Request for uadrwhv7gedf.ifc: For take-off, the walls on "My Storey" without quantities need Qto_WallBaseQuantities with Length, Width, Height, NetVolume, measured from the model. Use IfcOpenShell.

First a look at what the model holds.

```python
import ifcopenshell
import ifcopenshell.util.element
import ifcopenshell.util.unit

model = ifcopenshell.open("uadrwhv7gedf.ifc")
print(model.schema)
for unit_type in ("LENGTHUNIT", "AREAUNIT", "VOLUMEUNIT"):
    print(unit_type, ifcopenshell.util.unit.calculate_unit_scale(model, unit_type))
storey = next(s for s in model.by_type("IfcBuildingStorey") if s.Name == "My Storey")
walls = [e for e in ifcopenshell.util.element.get_decomposition(storey) if e.is_a("IfcWall")]
for e in sorted(walls, key=lambda e: e.id()):
    print(e.id(), e.is_a(), e.Name, list(ifcopenshell.util.element.get_psets(e, qtos_only=True)), sep=" | ")
```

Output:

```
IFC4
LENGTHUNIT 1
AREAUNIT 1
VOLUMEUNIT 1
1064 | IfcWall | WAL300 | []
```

```python
import ifcopenshell
import ifcopenshell.api.pset
import ifcopenshell.geom
import ifcopenshell.util.element
import ifcopenshell.util.shape
import ifcopenshell.util.unit

model = ifcopenshell.open("uadrwhv7gedf.ifc")
unit_scale = ifcopenshell.util.unit.calculate_unit_scale(model)
volume_scale = ifcopenshell.util.unit.calculate_unit_scale(model, "VOLUMEUNIT")
settings = ifcopenshell.geom.settings()

storey = next(s for s in model.by_type("IfcBuildingStorey") if s.Name == "My Storey")
walls = [e for e in ifcopenshell.util.element.get_decomposition(storey) if e.is_a("IfcWall")]

for e in sorted(walls, key=lambda e: e.id()):
    if ifcopenshell.util.element.get_psets(e, qtos_only=True, should_inherit=False):
        continue
    # Geometry comes back in metres, in the element's own axes.
    shape = ifcopenshell.geom.create_shape(settings, e)
    values = {
        "Length": ifcopenshell.util.shape.get_x(shape.geometry) / unit_scale,
        "Width": ifcopenshell.util.shape.get_y(shape.geometry) / unit_scale,
        "Height": ifcopenshell.util.shape.get_z(shape.geometry) / unit_scale,
        "NetVolume": ifcopenshell.util.shape.get_volume(shape.geometry) / volume_scale,
    }
    qto = ifcopenshell.api.pset.add_qto(model, product=e, name="Qto_WallBaseQuantities")
    ifcopenshell.api.pset.edit_qto(model, qto=qto, properties=values)
    print(e.id(), {k: round(v, 3) for k, v in values.items()})

model.write("uadrwhv7gedf_v2.ifc")
```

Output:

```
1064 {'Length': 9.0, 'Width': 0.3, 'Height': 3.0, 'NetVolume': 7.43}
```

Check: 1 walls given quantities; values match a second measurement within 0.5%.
